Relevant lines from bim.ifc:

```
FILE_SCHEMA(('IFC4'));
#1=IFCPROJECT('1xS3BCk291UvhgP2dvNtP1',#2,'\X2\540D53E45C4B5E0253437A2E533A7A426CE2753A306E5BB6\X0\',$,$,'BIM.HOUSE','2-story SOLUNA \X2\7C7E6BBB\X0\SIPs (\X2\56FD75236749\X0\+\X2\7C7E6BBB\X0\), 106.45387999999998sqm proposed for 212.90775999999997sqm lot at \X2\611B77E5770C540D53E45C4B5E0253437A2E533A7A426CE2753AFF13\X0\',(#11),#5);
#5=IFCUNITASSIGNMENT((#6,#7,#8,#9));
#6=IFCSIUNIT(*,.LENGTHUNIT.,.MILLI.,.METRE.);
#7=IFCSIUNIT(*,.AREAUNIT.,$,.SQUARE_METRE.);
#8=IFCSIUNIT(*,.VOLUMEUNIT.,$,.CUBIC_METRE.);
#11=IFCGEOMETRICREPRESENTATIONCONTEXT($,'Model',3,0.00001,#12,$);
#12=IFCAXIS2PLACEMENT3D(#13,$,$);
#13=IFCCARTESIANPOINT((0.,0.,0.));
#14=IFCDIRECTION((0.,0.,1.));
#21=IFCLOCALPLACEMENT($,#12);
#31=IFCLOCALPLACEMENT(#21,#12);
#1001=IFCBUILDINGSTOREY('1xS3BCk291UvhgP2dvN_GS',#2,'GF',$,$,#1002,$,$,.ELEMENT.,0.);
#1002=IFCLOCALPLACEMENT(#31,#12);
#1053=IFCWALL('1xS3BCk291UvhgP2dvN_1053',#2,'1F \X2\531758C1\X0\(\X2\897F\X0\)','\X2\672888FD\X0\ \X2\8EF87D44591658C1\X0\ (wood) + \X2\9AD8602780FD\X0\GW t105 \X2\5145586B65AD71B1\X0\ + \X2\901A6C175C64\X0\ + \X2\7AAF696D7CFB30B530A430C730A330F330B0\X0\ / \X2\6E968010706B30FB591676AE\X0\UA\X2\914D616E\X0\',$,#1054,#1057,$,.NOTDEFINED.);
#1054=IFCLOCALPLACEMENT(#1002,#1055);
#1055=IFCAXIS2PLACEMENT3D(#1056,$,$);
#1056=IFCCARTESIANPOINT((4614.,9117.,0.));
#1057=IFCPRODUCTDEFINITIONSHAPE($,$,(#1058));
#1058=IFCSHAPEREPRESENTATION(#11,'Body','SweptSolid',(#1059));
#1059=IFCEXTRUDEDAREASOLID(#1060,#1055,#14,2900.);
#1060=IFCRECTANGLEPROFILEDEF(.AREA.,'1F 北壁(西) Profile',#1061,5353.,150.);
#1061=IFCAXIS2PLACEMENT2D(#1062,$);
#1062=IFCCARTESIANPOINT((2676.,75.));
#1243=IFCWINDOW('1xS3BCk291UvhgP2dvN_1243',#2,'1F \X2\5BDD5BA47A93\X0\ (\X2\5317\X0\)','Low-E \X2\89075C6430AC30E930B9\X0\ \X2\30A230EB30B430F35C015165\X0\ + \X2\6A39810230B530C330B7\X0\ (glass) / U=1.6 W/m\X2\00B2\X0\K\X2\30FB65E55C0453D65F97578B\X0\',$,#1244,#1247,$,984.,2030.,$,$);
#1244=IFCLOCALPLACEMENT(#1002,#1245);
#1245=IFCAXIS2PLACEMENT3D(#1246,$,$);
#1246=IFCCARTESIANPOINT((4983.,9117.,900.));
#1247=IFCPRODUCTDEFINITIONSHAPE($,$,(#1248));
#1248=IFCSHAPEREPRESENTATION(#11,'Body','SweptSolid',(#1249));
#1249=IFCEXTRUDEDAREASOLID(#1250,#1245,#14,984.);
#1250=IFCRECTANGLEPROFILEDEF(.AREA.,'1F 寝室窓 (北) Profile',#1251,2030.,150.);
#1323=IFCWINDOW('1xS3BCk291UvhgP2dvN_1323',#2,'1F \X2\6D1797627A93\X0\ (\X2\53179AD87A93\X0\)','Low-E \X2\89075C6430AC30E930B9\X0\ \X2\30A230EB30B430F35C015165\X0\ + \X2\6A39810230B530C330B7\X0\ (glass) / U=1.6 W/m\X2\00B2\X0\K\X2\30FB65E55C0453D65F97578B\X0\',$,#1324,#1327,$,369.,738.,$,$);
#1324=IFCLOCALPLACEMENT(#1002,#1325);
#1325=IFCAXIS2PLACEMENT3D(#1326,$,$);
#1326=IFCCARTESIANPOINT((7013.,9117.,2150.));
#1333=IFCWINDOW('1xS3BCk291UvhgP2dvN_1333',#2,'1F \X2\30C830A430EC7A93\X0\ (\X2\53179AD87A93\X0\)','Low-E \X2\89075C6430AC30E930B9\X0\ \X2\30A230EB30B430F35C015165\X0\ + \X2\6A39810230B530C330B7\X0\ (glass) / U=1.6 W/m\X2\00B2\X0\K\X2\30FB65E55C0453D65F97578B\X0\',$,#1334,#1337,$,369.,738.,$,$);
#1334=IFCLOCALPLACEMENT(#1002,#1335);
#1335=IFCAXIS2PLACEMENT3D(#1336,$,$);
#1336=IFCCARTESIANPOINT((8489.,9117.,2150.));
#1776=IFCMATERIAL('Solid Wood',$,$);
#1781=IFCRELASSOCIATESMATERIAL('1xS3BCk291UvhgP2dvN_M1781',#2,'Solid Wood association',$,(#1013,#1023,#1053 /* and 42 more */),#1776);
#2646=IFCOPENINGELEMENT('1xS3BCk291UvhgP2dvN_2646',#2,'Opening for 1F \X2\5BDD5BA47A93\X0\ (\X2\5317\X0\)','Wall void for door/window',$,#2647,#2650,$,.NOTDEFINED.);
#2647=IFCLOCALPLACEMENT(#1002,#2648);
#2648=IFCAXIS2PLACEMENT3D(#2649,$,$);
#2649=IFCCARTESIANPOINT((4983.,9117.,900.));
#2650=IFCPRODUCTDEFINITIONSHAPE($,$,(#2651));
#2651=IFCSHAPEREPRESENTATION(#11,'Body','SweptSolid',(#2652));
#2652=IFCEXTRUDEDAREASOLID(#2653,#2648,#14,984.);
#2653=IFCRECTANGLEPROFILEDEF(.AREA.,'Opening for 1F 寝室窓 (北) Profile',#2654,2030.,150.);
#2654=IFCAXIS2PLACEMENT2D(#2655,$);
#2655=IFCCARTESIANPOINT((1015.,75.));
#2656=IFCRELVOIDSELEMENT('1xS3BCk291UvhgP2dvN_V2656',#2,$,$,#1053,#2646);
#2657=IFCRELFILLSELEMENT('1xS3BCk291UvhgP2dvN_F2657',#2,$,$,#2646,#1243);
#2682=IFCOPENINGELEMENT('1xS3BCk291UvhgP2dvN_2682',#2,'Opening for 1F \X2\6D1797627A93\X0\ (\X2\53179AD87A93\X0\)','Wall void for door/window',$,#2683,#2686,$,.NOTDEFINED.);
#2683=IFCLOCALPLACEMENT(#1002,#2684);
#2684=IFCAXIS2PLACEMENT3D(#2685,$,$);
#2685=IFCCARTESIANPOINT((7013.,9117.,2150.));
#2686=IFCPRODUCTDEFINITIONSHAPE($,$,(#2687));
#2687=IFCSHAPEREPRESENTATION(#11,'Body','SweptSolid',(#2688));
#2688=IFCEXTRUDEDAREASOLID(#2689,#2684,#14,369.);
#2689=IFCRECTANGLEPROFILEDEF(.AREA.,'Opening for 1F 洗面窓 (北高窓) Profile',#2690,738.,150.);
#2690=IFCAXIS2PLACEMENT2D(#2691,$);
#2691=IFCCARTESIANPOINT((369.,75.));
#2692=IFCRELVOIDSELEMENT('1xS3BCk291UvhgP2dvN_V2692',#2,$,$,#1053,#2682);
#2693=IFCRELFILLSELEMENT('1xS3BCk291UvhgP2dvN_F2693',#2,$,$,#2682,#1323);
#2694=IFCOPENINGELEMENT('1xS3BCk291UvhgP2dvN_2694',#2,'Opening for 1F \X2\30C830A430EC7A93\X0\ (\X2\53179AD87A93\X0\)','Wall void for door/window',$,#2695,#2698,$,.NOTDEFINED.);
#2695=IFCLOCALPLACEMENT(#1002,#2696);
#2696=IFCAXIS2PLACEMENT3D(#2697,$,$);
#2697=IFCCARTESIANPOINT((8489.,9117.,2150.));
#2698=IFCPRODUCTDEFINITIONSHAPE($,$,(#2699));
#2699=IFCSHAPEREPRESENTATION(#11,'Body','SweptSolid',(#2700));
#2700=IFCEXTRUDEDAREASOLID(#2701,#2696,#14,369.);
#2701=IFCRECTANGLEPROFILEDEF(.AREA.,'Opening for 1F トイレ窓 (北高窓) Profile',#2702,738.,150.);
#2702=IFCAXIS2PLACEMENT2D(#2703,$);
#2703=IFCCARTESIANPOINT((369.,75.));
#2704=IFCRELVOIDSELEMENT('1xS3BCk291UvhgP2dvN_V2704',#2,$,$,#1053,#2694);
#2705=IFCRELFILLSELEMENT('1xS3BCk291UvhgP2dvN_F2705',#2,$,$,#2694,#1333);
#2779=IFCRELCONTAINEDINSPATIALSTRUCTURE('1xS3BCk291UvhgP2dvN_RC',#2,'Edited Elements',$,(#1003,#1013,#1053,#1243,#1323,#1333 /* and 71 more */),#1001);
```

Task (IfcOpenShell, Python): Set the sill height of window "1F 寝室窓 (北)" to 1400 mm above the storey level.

```python
import numpy as np
import ifcopenshell
import ifcopenshell.api.geometry
import ifcopenshell.geom
import ifcopenshell.util.element
import ifcopenshell.util.placement
import ifcopenshell.util.shape
import ifcopenshell.util.unit

model = ifcopenshell.open("bim.ifc")
unit_scale = ifcopenshell.util.unit.calculate_unit_scale(model)

window = model.by_id(1243)
opening = window.FillsVoids[0].RelatingOpeningElement
storey = ifcopenshell.util.element.get_container(window, ifc_class="IfcBuildingStorey")
level = ifcopenshell.util.placement.get_local_placement(storey.ObjectPlacement)[2, 3]

# The opening's origin need not be at the sill, so measure its lowest point.
shape = ifcopenshell.geom.create_shape(ifcopenshell.geom.settings(), opening)
bottom = ifcopenshell.util.shape.get_shape_bottom_elevation(shape, shape.geometry) / unit_scale
dz = level + 1.4 / unit_scale - bottom

shift = np.array([0.0, 0.0, dz])
# The window is not placed relative to its opening, so move both.
for product in (opening, window):
    matrix = ifcopenshell.util.placement.get_local_placement(product.ObjectPlacement)
    matrix[:3, 3] += shift
    ifcopenshell.api.geometry.edit_object_placement(model, product=product, matrix=matrix, is_si=False)

print(f"moved by {dz * unit_scale:+.3f} m")

model.write("bim_v2.ifc")
```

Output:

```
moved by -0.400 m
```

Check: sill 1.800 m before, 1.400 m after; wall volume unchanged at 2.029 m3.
